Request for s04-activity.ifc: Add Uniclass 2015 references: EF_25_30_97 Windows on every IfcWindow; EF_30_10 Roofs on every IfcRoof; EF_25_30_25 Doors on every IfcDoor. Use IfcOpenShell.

First a look at what the model holds.

```python
import ifcopenshell

model = ifcopenshell.open("s04-activity.ifc")
print(model.schema)
print("classifications:", [c.Name for c in model.by_type("IfcClassification")])
for ifc_class in ("IfcDoor", "IfcRoof", "IfcStair", "IfcWall", "IfcWindow"):
    print(ifc_class, len(model.by_type(ifc_class)))
```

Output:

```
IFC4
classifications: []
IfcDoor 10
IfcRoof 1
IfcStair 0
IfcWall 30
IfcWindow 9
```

```python
import ifcopenshell
import ifcopenshell.api.classification

model = ifcopenshell.open("s04-activity.ifc")

system = ifcopenshell.api.classification.add_classification(model, classification="Uniclass 2015")

codes = {
    "IfcWindow": ("EF_25_30_97", "Windows"),
    "IfcRoof": ("EF_30_10", "Roofs"),
    "IfcDoor": ("EF_25_30_25", "Doors"),
}
for ifc_class, (code, name) in codes.items():
    products = model.by_type(ifc_class)
    ifcopenshell.api.classification.add_reference(
        model, products=products, classification=system, identification=code, name=name
    )
    print(code, len(products))

model.write("s04-activity_rev.ifc")
```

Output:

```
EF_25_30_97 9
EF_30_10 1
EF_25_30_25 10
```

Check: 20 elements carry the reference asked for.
